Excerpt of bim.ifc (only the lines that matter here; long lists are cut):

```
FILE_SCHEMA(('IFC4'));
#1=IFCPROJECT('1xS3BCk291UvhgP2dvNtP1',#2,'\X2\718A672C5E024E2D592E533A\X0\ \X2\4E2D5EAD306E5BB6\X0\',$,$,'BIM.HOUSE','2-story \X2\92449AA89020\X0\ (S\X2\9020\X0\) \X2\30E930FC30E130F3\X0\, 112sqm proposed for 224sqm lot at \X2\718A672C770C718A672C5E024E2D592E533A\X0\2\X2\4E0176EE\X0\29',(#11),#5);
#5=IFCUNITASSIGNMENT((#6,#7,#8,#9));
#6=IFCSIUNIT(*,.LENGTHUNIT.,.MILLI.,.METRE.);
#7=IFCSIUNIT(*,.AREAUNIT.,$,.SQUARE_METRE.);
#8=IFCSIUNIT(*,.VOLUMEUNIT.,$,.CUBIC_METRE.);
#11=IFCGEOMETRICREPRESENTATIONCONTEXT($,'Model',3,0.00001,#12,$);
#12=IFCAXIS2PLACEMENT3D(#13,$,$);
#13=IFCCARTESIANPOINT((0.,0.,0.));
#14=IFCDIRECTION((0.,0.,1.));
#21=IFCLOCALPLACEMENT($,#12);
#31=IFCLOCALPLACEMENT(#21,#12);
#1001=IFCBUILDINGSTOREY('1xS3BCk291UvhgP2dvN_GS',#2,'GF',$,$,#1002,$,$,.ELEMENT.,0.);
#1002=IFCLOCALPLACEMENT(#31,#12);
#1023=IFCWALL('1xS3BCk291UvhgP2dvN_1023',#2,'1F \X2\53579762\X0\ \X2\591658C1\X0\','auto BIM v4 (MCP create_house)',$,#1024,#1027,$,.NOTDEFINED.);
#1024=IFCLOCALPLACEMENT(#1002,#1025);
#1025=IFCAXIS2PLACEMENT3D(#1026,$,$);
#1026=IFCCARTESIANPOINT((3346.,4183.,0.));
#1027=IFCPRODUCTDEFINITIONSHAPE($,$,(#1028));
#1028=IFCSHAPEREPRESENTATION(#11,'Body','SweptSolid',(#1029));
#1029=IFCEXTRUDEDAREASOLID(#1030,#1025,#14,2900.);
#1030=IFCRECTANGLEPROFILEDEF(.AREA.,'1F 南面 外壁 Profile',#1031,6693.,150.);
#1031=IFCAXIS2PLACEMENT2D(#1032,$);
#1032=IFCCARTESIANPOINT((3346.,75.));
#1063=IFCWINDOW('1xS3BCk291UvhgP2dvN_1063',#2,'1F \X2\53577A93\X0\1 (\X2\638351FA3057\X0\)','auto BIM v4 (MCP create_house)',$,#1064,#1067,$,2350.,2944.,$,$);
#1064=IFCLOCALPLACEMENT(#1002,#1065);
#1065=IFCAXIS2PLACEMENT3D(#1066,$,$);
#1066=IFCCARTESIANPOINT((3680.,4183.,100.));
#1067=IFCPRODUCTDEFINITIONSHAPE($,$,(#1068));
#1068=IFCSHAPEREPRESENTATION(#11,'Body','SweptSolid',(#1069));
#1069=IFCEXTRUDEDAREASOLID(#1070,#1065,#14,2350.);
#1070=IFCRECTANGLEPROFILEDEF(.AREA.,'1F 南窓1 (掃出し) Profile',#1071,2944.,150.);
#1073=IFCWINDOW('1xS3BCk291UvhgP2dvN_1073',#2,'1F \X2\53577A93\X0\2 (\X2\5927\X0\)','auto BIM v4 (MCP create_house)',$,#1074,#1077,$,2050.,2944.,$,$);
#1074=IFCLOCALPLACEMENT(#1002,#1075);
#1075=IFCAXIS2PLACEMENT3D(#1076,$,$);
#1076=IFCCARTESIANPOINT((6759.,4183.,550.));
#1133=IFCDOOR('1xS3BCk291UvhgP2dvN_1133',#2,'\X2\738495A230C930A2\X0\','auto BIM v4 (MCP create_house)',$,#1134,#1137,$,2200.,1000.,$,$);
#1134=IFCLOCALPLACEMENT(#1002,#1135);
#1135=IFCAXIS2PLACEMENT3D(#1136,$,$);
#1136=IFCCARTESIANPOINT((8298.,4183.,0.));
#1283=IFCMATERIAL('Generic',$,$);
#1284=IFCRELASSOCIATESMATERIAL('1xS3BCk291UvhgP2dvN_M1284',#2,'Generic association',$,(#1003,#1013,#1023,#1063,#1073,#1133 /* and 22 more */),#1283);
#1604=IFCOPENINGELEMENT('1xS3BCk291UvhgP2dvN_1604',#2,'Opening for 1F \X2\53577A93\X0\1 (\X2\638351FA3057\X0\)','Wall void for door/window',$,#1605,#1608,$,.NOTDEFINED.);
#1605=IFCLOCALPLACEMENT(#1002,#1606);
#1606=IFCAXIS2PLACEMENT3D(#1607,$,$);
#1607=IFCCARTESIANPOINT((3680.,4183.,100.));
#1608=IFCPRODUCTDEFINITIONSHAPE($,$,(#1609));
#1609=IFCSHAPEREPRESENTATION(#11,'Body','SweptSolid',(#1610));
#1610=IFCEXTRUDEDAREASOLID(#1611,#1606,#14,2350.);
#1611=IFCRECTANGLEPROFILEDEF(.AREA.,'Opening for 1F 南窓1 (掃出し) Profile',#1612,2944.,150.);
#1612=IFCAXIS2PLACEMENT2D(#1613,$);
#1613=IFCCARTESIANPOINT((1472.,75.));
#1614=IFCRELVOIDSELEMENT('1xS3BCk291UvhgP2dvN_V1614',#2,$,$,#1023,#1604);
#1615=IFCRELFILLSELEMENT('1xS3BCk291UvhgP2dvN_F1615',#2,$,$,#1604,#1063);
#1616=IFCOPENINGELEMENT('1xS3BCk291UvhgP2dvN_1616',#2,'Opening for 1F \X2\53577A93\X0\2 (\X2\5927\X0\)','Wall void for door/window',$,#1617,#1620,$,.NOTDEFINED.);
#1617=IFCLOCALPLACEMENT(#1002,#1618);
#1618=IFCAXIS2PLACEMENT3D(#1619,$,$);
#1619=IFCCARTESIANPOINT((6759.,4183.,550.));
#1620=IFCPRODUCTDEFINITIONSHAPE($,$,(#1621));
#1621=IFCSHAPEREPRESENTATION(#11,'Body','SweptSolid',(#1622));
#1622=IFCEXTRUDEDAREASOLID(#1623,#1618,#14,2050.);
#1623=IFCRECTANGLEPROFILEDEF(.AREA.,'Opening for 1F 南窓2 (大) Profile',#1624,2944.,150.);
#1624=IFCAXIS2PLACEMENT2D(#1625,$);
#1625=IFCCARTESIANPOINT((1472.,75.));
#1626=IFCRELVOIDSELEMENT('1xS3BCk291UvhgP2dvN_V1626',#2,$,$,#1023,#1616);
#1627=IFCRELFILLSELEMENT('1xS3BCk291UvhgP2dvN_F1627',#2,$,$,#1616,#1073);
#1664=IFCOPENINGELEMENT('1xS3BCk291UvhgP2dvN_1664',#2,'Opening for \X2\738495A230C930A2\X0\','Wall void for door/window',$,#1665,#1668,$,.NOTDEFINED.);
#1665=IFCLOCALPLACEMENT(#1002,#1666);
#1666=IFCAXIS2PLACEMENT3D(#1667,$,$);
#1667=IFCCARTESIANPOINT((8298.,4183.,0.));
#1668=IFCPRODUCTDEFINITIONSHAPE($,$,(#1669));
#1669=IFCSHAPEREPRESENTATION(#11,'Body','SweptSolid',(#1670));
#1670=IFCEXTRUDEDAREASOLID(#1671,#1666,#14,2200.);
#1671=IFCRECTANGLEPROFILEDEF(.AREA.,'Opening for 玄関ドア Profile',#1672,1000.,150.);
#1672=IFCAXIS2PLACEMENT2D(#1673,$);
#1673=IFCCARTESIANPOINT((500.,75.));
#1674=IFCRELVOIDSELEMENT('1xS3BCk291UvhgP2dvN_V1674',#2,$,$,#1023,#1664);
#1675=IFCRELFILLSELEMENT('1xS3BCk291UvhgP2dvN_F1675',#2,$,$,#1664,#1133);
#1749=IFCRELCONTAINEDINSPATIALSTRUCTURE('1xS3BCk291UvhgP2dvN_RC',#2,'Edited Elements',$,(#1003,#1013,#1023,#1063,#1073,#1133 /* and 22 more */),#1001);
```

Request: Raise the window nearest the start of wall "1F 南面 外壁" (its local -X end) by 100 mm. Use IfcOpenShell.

```python
import numpy as np
import ifcopenshell
import ifcopenshell.api.geometry
import ifcopenshell.util.placement
import ifcopenshell.util.unit

model = ifcopenshell.open("bim.ifc")
unit_scale = ifcopenshell.util.unit.calculate_unit_scale(model)

window = model.by_guid("1xS3BCk291UvhgP2dvN_1063")
opening = window.FillsVoids[0].RelatingOpeningElement
dz = 0.1 / unit_scale

shift = np.array([0.0, 0.0, dz])
# The window is not placed relative to its opening, so move both.
for product in (opening, window):
    matrix = ifcopenshell.util.placement.get_local_placement(product.ObjectPlacement)
    matrix[:3, 3] += shift
    ifcopenshell.api.geometry.edit_object_placement(model, product=product, matrix=matrix, is_si=False)

print(f"moved by {dz * unit_scale:+.3f} m")

model.write("bim-out.ifc")
```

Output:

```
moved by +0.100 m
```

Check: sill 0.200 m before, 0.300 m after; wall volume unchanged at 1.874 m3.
